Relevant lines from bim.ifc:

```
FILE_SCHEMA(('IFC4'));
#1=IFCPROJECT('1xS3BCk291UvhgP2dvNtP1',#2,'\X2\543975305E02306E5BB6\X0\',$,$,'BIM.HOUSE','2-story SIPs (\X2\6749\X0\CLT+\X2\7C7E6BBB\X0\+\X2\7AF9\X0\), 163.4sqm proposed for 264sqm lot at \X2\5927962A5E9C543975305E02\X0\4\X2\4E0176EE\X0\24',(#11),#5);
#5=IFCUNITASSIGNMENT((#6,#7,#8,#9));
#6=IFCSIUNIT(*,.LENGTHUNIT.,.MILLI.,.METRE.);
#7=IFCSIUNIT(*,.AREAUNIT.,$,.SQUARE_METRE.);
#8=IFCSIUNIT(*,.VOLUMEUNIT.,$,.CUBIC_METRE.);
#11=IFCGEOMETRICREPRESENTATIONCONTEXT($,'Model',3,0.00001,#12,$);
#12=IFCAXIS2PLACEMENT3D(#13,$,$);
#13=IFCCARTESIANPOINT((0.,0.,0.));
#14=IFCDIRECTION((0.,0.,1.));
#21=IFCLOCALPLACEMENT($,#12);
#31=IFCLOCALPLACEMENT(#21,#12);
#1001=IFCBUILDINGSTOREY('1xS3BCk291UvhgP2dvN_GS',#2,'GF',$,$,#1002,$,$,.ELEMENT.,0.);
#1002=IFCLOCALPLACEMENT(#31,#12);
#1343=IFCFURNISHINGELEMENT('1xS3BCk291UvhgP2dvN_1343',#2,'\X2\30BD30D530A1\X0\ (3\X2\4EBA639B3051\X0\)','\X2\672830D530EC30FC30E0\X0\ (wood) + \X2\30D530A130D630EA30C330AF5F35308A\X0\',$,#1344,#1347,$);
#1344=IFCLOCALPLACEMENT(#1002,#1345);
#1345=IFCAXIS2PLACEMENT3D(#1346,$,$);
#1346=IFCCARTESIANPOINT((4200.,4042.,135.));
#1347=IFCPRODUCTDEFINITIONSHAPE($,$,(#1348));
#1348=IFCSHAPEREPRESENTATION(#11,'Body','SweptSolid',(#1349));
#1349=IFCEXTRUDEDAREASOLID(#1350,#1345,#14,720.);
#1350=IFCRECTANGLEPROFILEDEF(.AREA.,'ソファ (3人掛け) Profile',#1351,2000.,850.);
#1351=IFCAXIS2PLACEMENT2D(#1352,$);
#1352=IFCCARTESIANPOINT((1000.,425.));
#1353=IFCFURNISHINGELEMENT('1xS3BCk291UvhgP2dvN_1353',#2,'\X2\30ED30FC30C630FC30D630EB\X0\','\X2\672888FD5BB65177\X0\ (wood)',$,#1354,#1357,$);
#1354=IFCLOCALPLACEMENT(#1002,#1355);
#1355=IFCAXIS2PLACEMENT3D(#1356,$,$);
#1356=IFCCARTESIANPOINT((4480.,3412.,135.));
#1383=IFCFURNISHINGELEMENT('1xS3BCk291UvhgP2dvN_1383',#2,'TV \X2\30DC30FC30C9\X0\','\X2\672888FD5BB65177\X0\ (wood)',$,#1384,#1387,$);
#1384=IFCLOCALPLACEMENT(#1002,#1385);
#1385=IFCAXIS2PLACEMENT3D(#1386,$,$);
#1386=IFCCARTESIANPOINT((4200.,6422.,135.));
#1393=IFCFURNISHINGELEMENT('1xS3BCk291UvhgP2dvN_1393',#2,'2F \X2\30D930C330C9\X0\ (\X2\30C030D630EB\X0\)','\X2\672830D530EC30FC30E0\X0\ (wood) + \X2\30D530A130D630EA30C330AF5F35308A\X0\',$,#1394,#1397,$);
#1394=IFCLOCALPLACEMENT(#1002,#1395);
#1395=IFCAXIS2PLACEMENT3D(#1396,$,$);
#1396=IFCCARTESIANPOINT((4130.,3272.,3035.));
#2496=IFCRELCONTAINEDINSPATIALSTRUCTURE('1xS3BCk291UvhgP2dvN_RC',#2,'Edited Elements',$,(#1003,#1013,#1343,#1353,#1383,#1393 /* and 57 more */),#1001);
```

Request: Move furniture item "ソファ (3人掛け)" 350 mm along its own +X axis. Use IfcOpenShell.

```python
import ifcopenshell
import ifcopenshell.api.geometry
import ifcopenshell.util.placement
import ifcopenshell.util.unit

model = ifcopenshell.open("bim.ifc")
unit_scale = ifcopenshell.util.unit.calculate_unit_scale(model)

item = model.by_guid("1xS3BCk291UvhgP2dvN_1343")
matrix = ifcopenshell.util.placement.get_local_placement(item.ObjectPlacement)
matrix[:3, 3] += matrix[:3, 0] * 0.35 / unit_scale
ifcopenshell.api.geometry.edit_object_placement(model, product=item, matrix=matrix, is_si=False)

print(ifcopenshell.util.placement.get_local_placement(item.ObjectPlacement).round(3) + 0.0)

model.write("bim_v2.ifc")
```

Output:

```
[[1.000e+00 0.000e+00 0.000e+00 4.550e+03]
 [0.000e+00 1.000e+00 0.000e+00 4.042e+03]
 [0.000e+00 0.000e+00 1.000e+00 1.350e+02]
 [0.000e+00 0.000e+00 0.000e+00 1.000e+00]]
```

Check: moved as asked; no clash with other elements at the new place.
